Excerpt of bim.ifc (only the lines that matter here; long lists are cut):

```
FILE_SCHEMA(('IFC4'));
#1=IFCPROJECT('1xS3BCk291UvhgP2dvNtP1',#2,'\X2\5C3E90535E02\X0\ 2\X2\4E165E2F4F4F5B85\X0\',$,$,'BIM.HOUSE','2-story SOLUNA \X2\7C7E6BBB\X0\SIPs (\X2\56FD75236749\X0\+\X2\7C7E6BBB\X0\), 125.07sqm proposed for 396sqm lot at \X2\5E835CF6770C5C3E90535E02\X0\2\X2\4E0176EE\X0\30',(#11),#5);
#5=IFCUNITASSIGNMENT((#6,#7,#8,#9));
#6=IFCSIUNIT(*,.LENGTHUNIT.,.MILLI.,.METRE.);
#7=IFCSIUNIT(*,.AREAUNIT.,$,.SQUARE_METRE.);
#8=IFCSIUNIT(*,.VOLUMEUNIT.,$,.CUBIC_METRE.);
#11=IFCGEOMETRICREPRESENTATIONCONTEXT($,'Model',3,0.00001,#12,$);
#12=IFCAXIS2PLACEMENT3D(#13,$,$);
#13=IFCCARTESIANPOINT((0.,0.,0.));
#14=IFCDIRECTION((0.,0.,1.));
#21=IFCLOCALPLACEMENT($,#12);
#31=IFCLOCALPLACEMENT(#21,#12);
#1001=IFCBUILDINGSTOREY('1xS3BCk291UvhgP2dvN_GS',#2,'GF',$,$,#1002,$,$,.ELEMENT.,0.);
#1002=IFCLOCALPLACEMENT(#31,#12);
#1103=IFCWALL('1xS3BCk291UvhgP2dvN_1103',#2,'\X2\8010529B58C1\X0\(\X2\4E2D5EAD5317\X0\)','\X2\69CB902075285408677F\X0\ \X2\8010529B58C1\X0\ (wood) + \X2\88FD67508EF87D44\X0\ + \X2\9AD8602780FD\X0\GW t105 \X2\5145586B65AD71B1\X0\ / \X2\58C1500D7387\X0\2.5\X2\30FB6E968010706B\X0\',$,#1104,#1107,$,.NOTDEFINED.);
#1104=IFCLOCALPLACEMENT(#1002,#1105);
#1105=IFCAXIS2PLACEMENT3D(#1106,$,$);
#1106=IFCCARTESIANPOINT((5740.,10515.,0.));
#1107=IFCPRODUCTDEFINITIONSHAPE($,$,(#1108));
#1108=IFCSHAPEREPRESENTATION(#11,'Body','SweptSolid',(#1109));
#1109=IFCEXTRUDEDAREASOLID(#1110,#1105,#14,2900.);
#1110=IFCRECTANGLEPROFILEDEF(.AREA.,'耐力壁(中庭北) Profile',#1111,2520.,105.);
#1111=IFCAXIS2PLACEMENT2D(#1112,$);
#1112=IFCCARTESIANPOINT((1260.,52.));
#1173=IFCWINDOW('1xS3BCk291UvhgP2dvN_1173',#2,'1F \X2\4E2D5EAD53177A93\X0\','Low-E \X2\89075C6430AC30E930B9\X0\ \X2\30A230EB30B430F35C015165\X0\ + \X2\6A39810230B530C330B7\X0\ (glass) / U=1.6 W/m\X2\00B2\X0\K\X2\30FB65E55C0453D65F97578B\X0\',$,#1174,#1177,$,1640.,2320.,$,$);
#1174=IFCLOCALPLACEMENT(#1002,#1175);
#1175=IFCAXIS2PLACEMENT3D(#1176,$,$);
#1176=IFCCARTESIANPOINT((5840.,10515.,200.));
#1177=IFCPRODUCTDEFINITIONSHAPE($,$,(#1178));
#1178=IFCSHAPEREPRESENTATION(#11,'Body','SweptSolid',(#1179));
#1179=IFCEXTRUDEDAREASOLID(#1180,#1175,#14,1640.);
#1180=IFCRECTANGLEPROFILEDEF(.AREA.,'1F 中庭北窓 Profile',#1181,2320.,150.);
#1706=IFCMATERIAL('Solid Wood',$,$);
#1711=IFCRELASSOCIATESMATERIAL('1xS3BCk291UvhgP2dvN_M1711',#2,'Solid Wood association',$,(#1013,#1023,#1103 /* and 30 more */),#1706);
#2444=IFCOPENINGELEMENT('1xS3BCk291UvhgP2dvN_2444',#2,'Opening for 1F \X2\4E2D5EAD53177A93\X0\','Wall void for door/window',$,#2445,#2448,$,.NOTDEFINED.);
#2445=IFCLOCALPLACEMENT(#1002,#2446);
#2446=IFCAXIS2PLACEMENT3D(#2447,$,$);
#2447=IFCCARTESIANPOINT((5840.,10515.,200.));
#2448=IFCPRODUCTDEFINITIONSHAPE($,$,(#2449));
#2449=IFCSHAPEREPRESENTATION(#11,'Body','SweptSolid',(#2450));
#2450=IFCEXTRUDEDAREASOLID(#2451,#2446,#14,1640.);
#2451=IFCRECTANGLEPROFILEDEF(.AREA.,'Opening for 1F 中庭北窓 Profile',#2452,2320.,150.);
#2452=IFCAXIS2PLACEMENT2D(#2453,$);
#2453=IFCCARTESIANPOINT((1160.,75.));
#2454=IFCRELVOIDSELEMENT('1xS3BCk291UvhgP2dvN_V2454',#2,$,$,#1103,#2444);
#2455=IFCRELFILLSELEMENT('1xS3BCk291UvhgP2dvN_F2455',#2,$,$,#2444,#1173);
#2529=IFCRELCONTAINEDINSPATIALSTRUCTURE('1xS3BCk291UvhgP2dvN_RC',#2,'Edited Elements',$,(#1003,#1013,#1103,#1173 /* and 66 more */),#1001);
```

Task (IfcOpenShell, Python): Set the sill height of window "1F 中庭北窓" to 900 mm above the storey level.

```python
import numpy as np
import ifcopenshell
import ifcopenshell.api.geometry
import ifcopenshell.geom
import ifcopenshell.util.element
import ifcopenshell.util.placement
import ifcopenshell.util.shape
import ifcopenshell.util.unit

model = ifcopenshell.open("bim.ifc")
unit_scale = ifcopenshell.util.unit.calculate_unit_scale(model)

window = model.by_guid("1xS3BCk291UvhgP2dvN_1173")
opening = window.FillsVoids[0].RelatingOpeningElement
storey = ifcopenshell.util.element.get_container(window, ifc_class="IfcBuildingStorey")
level = ifcopenshell.util.placement.get_local_placement(storey.ObjectPlacement)[2, 3]

# The opening's origin need not be at the sill, so measure its lowest point.
shape = ifcopenshell.geom.create_shape(ifcopenshell.geom.settings(), opening)
bottom = ifcopenshell.util.shape.get_shape_bottom_elevation(shape, shape.geometry) / unit_scale
dz = level + 900.0 - bottom

shift = np.array([0.0, 0.0, dz])
# The window is not placed relative to its opening, so move both.
for product in (opening, window):
    matrix = ifcopenshell.util.placement.get_local_placement(product.ObjectPlacement)
    matrix[:3, 3] += shift
    ifcopenshell.api.geometry.edit_object_placement(model, product=product, matrix=matrix, is_si=False)

print(f"moved by {dz * unit_scale:+.3f} m")

model.write("bim_updated.ifc")
```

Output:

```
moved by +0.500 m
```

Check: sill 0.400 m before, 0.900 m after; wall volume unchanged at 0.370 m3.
